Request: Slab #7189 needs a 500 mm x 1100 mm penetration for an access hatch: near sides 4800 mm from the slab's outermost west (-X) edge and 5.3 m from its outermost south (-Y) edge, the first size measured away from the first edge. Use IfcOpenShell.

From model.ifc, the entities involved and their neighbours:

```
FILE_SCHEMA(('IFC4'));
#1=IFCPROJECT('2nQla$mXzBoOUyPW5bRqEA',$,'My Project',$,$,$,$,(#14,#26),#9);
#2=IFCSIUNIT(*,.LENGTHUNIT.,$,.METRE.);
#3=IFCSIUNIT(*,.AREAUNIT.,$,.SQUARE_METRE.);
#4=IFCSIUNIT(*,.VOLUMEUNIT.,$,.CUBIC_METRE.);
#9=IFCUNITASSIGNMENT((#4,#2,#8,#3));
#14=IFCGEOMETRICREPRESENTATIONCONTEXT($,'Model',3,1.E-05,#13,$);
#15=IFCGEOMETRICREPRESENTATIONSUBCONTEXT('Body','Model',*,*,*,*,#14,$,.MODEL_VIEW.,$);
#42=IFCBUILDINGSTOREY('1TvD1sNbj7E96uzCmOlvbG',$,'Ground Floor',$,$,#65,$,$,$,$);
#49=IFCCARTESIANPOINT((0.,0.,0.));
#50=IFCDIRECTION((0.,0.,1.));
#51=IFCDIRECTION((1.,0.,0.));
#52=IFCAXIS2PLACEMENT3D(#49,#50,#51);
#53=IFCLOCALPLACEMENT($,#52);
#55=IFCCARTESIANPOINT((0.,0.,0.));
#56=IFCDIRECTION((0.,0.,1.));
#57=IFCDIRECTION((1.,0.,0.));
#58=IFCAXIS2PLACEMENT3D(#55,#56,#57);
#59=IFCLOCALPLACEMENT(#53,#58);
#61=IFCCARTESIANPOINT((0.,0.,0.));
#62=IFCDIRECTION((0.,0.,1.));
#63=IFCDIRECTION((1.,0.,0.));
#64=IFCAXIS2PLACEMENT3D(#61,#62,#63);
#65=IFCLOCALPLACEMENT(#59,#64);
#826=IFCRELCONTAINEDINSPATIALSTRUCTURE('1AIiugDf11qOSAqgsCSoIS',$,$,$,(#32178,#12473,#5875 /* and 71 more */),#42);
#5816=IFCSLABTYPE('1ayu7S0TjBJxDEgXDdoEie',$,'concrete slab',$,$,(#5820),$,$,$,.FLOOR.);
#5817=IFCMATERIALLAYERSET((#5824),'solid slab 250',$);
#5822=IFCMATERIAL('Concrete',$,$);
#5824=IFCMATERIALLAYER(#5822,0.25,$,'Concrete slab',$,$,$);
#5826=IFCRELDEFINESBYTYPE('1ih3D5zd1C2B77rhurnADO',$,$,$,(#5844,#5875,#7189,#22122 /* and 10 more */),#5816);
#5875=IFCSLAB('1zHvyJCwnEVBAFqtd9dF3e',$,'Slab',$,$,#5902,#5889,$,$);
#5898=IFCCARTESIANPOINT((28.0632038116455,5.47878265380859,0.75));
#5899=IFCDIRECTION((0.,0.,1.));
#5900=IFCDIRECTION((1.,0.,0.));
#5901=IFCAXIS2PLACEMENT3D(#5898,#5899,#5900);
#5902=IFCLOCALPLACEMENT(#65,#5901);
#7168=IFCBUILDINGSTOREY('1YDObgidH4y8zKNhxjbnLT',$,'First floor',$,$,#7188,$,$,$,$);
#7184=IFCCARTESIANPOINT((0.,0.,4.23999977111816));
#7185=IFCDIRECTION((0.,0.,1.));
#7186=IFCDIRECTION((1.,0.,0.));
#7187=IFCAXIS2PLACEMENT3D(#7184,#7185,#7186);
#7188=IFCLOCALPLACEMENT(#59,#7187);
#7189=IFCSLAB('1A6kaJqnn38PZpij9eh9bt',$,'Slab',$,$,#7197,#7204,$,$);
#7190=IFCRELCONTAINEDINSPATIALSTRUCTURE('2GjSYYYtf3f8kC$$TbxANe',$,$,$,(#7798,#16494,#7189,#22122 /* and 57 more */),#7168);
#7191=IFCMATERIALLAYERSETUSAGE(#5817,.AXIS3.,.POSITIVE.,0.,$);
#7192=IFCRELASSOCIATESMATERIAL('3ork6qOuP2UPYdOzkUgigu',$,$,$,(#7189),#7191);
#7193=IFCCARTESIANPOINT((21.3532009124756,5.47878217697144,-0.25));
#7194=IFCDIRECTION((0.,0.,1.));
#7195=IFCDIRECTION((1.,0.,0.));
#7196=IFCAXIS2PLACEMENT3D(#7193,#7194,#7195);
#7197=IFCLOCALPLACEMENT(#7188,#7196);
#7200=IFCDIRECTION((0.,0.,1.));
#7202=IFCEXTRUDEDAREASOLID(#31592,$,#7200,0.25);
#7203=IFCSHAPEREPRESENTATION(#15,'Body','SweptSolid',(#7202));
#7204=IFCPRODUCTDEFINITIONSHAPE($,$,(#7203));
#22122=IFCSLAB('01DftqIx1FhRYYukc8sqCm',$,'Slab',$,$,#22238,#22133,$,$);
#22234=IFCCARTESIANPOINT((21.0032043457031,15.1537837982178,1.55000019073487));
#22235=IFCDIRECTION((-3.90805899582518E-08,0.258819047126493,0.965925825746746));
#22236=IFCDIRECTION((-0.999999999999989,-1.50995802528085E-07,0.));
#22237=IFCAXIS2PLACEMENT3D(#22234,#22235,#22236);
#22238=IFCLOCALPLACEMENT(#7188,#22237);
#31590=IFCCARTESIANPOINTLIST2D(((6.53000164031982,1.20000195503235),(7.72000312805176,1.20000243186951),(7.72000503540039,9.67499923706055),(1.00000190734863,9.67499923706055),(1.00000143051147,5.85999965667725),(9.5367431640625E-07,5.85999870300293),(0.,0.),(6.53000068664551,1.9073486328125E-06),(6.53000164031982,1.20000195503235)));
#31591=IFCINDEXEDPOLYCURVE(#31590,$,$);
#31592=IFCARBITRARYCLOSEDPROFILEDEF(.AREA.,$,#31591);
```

```python
import numpy as np
import ifcopenshell
import ifcopenshell.api.feature
import ifcopenshell.api.geometry
import ifcopenshell.api.root
import ifcopenshell.geom
import ifcopenshell.util.placement
import ifcopenshell.util.representation
import ifcopenshell.util.shape
import ifcopenshell.util.unit

model = ifcopenshell.open("model.ifc")
unit_scale = ifcopenshell.util.unit.calculate_unit_scale(model)
settings = ifcopenshell.geom.settings()


def volume(element):
    """Net volume in cubic metres, openings subtracted."""
    shape = ifcopenshell.geom.create_shape(settings, element)
    return ifcopenshell.util.shape.get_volume(shape.geometry)


slab = model.by_id(7189)
before = volume(slab)

# Extent in the slab's own axes, in metres. The edges named are its -X and -Y sides.
slab_shape = ifcopenshell.geom.create_shape(settings, slab)
vertices = ifcopenshell.util.shape.get_vertices(slab_shape.geometry)
x_min, y_min, bottom = vertices.min(axis=0)
top = vertices[:, 2].max()

opening = ifcopenshell.api.root.create_entity(model, ifc_class="IfcOpeningElement", name="Access hatch opening", predefined_type="OPENING")
context = ifcopenshell.util.representation.get_context(model, "Model", "Body", "MODEL_VIEW")
width, depth = 0.5, 1.1
outline = [(0.0, 0.0), (width, 0.0), (width, depth), (0.0, depth), (0.0, 0.0)]
# Overshoot both faces by 50 mm so the cut is clean.
shape = ifcopenshell.api.geometry.add_slab_representation(
    model, context=context, depth=top - bottom + 0.1, polyline=outline
)
ifcopenshell.api.geometry.assign_representation(model, product=opening, representation=shape)

matrix = ifcopenshell.util.placement.get_local_placement(slab.ObjectPlacement)
matrix[:, 3] = matrix @ np.append(np.array([x_min + 4.8, y_min + 5.3, bottom - 0.05]) / unit_scale, 1.0)
ifcopenshell.api.geometry.edit_object_placement(model, product=opening, matrix=matrix, is_si=False)
ifcopenshell.api.feature.add_feature(model, feature=opening, element=slab)

after = volume(slab)

print(f"slab volume {before:.3f} -> {after:.3f} m3")

model.write("model_updated.ifc")
```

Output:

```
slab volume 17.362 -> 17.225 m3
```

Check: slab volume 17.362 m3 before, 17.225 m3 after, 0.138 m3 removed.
